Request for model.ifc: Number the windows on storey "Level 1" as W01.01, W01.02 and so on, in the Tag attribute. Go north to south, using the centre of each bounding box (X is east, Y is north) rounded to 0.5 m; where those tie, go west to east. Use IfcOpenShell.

First a look at what the model holds.

```python
import ifcopenshell
import ifcopenshell.util.element
import ifcopenshell.util.placement

model = ifcopenshell.open("model.ifc")
print(model.schema)
storey = next(s for s in model.by_type("IfcBuildingStorey") if s.Name == "Level 1")
windows = [e for e in ifcopenshell.util.element.get_decomposition(storey) if e.is_a("IfcWindow")]
for e in sorted(windows, key=lambda e: e.id()):
    origin = ifcopenshell.util.placement.get_local_placement(e.ObjectPlacement)[:3, 3]
    print(e.id(), e.Tag, e.Name, origin.round(2) + 0.0, sep=" | ")
```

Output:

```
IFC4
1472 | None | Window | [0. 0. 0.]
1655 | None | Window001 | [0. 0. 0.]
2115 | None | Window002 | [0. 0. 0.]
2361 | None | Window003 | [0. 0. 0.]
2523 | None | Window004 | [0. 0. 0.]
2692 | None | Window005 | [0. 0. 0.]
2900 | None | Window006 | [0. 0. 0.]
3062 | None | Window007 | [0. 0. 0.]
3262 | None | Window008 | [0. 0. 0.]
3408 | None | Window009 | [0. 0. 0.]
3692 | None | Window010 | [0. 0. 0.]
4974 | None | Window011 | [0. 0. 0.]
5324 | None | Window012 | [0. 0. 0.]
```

```python
import ifcopenshell
import ifcopenshell.geom
import ifcopenshell.util.element
import ifcopenshell.util.shape

model = ifcopenshell.open("model.ifc")
settings = ifcopenshell.geom.settings()
settings.set("use-world-coords", True)


def centre(element):
    shape = ifcopenshell.geom.create_shape(settings, element)
    return ifcopenshell.util.shape.get_bbox_centroid(shape.geometry)


storey = next(s for s in model.by_type("IfcBuildingStorey") if s.Name == "Level 1")
windows = [e for e in ifcopenshell.util.element.get_decomposition(storey) if e.is_a("IfcWindow")]

# Insertion points can sit at a corner or the storey origin, so sort by the geometry (in metres).
centres = {e: centre(e) for e in windows}
windows.sort(key=lambda e: (-round(centres[e][1] / 0.5), centres[e][0]))

for i, e in enumerate(windows, start=1):
    number = f"W01.{i:02d}"
    e.Tag = number
    print(e.id(), number)

model.write("model_v2.ifc")
```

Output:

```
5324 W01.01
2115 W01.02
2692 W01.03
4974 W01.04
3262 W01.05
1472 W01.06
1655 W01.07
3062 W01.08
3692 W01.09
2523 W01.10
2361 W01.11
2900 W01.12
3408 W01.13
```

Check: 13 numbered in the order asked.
